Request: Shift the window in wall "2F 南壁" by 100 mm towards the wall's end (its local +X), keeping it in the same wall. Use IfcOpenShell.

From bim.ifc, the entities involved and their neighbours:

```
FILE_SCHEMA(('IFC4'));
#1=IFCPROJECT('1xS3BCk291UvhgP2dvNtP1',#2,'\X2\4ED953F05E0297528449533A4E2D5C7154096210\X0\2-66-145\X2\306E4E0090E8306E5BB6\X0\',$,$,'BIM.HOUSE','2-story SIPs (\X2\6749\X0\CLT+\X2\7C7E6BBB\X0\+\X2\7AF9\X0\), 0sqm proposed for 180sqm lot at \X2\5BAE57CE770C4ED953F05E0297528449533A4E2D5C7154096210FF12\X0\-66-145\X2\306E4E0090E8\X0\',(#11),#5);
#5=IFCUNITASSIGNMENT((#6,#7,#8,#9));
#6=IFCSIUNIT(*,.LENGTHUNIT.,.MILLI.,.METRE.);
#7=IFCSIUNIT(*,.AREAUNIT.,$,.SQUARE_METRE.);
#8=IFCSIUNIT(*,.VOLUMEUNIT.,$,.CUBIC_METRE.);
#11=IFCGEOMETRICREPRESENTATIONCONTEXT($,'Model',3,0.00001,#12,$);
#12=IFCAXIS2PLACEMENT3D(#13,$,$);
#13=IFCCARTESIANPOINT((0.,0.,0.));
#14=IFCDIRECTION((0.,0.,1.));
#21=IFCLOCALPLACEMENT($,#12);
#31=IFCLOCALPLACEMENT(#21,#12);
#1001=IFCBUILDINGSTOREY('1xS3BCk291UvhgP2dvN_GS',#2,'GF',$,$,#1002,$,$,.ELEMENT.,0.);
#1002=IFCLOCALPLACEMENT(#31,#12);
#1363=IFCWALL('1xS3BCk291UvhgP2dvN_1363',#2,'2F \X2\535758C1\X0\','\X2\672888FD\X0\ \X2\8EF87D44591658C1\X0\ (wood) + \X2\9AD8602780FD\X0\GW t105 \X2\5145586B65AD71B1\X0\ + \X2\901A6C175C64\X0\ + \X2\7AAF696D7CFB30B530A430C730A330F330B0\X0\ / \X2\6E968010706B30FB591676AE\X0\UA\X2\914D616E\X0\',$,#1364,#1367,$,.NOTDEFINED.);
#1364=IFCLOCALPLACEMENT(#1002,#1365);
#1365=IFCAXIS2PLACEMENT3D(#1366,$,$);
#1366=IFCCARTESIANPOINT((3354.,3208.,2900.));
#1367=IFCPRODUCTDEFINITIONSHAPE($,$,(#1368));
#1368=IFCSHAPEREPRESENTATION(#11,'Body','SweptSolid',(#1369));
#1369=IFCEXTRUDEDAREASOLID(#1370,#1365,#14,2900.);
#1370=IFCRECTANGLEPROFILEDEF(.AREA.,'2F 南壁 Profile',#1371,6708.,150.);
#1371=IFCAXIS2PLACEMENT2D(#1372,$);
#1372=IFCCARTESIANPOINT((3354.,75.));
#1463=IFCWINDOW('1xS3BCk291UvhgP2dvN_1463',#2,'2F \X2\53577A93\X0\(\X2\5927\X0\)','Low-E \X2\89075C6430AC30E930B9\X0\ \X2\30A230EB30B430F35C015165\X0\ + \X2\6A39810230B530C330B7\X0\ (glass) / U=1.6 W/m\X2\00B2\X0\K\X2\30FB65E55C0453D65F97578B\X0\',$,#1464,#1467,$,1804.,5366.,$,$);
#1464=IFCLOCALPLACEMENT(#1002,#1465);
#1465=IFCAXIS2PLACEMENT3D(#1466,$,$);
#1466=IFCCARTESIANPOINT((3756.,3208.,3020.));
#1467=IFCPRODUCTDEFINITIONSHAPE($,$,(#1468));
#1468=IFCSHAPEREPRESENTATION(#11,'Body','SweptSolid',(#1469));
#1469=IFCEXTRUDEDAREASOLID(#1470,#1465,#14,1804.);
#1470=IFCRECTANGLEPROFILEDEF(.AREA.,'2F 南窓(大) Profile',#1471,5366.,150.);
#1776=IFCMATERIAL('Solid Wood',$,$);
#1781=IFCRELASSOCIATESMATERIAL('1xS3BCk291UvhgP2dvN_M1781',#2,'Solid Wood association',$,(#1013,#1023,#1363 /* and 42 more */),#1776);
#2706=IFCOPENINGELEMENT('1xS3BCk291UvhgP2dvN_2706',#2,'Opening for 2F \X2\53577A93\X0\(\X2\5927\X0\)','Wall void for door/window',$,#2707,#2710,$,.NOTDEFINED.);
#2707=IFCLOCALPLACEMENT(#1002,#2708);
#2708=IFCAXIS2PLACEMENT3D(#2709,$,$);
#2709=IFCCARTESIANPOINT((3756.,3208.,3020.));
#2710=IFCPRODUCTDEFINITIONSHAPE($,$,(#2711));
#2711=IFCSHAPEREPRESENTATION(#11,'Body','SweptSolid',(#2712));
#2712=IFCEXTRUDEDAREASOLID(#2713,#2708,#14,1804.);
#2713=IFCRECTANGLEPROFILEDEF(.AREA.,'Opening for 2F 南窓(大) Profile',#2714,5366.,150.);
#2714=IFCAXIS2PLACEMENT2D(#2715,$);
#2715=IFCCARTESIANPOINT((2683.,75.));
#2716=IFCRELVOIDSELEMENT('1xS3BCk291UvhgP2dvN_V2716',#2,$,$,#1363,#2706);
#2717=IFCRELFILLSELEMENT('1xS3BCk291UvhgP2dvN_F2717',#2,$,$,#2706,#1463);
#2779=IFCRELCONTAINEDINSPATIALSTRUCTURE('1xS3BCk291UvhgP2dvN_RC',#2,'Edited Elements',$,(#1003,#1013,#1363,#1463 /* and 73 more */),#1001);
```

```python
import ifcopenshell
import ifcopenshell.api.geometry
import ifcopenshell.util.placement
import ifcopenshell.util.unit

model = ifcopenshell.open("bim.ifc")
unit_scale = ifcopenshell.util.unit.calculate_unit_scale(model)

window = model.by_id(1463)
opening = window.FillsVoids[0].RelatingOpeningElement
wall = opening.VoidsElements[0].RelatingBuildingElement

wall_matrix = ifcopenshell.util.placement.get_local_placement(wall.ObjectPlacement)
shift = wall_matrix[:3, 0] * 0.1 / unit_scale
before = ifcopenshell.util.placement.get_local_placement(window.ObjectPlacement)[:3, 3].copy()

# The window is not placed relative to its opening, so move both.
for product in (opening, window):
    matrix = ifcopenshell.util.placement.get_local_placement(product.ObjectPlacement)
    matrix[:3, 3] += shift
    ifcopenshell.api.geometry.edit_object_placement(model, product=product, matrix=matrix, is_si=False)

after = ifcopenshell.util.placement.get_local_placement(window.ObjectPlacement)[:3, 3]
print("window moved by", (after - before).round(3) + 0.0)

model.write("bim_updated.ifc")
```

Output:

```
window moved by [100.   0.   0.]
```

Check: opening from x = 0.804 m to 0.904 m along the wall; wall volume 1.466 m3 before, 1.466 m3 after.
